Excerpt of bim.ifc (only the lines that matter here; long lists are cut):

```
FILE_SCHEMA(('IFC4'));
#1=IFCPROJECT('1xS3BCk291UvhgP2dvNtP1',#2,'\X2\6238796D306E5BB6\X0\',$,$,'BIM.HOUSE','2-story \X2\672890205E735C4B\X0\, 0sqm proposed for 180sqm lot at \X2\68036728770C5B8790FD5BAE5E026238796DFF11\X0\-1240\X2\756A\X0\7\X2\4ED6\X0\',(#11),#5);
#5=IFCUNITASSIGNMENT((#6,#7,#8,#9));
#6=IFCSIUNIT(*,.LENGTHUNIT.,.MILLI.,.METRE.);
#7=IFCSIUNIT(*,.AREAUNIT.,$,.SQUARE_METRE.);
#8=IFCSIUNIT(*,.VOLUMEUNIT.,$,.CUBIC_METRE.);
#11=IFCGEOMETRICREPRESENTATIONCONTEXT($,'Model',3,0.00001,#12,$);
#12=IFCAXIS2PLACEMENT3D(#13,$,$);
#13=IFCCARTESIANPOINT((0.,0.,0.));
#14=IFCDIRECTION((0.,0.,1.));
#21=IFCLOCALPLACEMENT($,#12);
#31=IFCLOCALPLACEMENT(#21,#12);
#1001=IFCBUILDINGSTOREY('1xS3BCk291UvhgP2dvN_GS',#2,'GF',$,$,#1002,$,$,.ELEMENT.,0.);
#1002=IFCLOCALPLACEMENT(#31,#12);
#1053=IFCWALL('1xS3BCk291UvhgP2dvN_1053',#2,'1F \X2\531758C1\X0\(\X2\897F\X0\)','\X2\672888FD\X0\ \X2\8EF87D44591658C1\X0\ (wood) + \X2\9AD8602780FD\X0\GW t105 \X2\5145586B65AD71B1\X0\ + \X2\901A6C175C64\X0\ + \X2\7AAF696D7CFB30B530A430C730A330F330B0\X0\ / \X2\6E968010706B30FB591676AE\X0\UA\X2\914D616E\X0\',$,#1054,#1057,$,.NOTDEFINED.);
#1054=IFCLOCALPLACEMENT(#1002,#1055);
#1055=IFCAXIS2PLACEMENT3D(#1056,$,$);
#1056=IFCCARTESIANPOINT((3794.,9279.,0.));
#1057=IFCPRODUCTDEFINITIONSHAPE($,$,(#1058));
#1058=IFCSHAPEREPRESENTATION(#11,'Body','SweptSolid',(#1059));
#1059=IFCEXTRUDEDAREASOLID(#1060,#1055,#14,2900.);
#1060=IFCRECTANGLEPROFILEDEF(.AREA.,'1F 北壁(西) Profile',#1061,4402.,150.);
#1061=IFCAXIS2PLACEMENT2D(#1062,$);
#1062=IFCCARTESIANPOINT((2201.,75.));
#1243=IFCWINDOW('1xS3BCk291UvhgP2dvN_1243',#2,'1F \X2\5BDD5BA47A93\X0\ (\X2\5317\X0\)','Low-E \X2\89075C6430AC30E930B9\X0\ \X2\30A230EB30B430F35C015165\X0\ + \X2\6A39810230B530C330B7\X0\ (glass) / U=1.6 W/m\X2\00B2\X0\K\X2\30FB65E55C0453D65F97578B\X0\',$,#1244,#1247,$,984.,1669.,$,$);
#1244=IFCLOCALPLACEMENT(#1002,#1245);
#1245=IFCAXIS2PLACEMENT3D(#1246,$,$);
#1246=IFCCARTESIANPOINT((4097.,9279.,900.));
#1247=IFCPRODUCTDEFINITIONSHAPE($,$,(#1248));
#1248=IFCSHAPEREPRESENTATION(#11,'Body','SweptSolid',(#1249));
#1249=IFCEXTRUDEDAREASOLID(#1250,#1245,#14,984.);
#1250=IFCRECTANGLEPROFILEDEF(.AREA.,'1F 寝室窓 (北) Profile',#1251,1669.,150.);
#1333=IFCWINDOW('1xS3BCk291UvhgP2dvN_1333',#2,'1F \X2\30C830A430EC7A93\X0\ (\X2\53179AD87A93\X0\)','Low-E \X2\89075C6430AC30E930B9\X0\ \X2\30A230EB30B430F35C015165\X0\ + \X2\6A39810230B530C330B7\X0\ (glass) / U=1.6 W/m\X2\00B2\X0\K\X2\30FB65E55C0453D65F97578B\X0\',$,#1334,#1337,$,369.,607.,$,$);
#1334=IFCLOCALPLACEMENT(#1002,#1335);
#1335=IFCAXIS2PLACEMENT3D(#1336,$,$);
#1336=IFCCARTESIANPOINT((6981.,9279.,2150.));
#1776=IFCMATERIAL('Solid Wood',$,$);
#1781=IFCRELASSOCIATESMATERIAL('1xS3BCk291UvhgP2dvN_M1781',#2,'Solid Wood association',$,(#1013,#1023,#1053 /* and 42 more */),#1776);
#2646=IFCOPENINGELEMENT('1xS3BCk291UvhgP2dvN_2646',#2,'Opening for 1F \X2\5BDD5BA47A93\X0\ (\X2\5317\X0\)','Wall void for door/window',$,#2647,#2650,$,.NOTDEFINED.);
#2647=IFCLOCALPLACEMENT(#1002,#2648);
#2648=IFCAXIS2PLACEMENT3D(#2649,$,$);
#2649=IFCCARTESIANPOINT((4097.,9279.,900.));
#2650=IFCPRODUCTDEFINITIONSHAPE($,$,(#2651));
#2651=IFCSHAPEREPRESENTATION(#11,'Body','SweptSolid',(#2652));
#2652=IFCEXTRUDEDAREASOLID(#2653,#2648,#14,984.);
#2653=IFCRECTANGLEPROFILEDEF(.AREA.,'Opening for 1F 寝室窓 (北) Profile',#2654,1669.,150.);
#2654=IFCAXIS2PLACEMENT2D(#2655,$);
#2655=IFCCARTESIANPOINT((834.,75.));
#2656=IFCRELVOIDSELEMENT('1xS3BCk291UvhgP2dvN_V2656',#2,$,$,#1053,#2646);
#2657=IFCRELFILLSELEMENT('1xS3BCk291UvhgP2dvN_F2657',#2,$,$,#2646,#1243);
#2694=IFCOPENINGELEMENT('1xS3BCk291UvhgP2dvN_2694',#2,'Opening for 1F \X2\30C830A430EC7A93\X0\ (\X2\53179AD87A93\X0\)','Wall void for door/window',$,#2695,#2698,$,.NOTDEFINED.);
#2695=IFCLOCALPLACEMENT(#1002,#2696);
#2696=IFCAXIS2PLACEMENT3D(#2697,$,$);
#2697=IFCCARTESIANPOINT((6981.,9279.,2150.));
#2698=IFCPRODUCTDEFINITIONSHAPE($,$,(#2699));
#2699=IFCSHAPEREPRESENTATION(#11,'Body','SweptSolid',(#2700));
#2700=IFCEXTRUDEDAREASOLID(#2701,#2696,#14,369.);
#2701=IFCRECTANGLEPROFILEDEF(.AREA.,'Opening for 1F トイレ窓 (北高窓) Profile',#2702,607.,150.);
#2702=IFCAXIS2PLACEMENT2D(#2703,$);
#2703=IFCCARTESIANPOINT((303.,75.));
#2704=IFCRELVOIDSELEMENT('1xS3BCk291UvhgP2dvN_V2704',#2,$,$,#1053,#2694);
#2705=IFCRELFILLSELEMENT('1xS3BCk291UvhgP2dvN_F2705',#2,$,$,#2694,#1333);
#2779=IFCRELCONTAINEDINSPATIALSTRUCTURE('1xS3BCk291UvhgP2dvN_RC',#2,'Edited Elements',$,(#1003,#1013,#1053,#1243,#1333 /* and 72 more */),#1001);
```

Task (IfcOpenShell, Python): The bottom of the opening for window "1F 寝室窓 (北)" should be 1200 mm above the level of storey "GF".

```python
import numpy as np
import ifcopenshell
import ifcopenshell.api.geometry
import ifcopenshell.geom
import ifcopenshell.util.element
import ifcopenshell.util.placement
import ifcopenshell.util.shape
import ifcopenshell.util.unit

model = ifcopenshell.open("bim.ifc")
unit_scale = ifcopenshell.util.unit.calculate_unit_scale(model)

window = model.by_id(1243)
opening = window.FillsVoids[0].RelatingOpeningElement
storey = ifcopenshell.util.element.get_container(window, ifc_class="IfcBuildingStorey")
level = ifcopenshell.util.placement.get_local_placement(storey.ObjectPlacement)[2, 3]

# The opening's origin need not be at the sill, so measure its lowest point.
shape = ifcopenshell.geom.create_shape(ifcopenshell.geom.settings(), opening)
bottom = ifcopenshell.util.shape.get_shape_bottom_elevation(shape, shape.geometry) / unit_scale
dz = level + 1200.0 - bottom

shift = np.array([0.0, 0.0, dz])
# The window is not placed relative to its opening, so move both.
for product in (opening, window):
    matrix = ifcopenshell.util.placement.get_local_placement(product.ObjectPlacement)
    matrix[:3, 3] += shift
    ifcopenshell.api.geometry.edit_object_placement(model, product=product, matrix=matrix, is_si=False)

print(f"moved by {dz * unit_scale:+.3f} m")

model.write("bim-out.ifc")
```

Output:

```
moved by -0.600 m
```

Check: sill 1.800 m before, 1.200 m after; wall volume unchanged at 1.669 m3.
